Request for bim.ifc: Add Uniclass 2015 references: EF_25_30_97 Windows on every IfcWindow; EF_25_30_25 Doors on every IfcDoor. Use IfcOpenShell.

First a look at what the model holds.

```python
import ifcopenshell

model = ifcopenshell.open("bim.ifc")
print(model.schema)
print("classifications:", [c.Name for c in model.by_type("IfcClassification")])
for ifc_class in ("IfcDoor", "IfcRoof", "IfcStair", "IfcWall", "IfcWindow"):
    print(ifc_class, len(model.by_type(ifc_class)))
```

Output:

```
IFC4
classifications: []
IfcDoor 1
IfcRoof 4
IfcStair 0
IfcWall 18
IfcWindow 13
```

```python
import ifcopenshell
import ifcopenshell.api.classification

model = ifcopenshell.open("bim.ifc")

system = ifcopenshell.api.classification.add_classification(model, classification="Uniclass 2015")

codes = {
    "IfcWindow": ("EF_25_30_97", "Windows"),
    "IfcDoor": ("EF_25_30_25", "Doors"),
}
for ifc_class, (code, name) in codes.items():
    products = model.by_type(ifc_class)
    ifcopenshell.api.classification.add_reference(
        model, products=products, classification=system, identification=code, name=name
    )
    print(code, len(products))

model.write("bim_edited.ifc")
```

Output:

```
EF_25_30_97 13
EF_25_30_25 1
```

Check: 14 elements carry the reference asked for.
